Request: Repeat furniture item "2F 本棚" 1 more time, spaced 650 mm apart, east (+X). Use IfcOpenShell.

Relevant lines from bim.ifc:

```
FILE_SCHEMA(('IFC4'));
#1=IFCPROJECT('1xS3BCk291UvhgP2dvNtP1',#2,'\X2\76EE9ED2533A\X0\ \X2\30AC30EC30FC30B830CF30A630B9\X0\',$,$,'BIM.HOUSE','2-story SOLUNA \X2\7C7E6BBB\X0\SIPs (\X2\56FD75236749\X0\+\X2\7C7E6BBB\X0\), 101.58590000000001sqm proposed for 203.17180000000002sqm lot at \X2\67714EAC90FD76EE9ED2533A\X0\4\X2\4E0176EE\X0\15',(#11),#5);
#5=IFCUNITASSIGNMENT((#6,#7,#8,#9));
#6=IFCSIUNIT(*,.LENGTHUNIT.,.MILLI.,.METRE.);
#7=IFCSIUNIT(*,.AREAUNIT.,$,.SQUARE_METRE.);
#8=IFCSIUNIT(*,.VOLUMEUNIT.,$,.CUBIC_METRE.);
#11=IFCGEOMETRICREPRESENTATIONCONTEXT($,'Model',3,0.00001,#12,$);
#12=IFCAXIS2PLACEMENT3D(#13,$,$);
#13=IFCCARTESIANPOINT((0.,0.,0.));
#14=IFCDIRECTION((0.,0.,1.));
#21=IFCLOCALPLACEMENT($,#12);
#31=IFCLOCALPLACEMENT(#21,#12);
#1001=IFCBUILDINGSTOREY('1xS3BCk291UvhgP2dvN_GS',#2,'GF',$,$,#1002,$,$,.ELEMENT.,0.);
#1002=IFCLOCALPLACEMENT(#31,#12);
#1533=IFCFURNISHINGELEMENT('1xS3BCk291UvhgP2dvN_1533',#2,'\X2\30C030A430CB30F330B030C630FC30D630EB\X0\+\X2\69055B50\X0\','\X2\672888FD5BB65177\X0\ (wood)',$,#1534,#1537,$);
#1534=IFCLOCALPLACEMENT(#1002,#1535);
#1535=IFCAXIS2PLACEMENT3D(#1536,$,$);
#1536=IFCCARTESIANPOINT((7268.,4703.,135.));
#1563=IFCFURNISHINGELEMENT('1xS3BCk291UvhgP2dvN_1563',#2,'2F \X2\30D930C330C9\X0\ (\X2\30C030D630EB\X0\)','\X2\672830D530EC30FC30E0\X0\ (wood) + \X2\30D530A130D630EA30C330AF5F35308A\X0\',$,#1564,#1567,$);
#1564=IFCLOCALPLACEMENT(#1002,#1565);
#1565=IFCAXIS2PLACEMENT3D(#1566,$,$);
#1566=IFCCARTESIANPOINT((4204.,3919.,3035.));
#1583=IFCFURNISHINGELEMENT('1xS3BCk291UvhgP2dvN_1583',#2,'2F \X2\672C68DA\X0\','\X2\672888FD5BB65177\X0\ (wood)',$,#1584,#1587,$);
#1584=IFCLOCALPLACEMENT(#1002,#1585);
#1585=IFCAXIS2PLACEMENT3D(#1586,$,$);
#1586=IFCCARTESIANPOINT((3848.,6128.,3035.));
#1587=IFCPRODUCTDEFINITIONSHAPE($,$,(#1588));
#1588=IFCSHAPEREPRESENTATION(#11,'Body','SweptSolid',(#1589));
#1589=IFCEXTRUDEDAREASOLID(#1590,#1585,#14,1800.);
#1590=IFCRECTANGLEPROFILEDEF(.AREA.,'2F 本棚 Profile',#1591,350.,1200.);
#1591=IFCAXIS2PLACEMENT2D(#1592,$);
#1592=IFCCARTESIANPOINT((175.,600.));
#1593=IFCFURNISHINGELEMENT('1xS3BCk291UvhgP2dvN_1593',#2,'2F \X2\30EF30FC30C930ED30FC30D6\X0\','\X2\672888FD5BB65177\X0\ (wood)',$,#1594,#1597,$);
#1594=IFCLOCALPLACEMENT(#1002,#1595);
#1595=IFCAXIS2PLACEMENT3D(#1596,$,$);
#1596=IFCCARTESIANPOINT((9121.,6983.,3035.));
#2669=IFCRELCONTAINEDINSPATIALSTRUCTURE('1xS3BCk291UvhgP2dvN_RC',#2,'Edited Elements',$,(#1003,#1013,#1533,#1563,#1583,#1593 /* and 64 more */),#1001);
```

```python
import numpy as np
import ifcopenshell
import ifcopenshell.api.geometry
import ifcopenshell.api.root
import ifcopenshell.util.element
import ifcopenshell.util.placement

model = ifcopenshell.open("bim.ifc")


def reuse_history(source, copy):
    """copy_class also copies each property set's owner history, people and application; keep the originals."""
    for rel in copy.IsDefinedBy:
        if rel.is_a("IfcRelDefinesByProperties") and (history := rel.RelatingPropertyDefinition.OwnerHistory):
            rel.RelatingPropertyDefinition.OwnerHistory = source.OwnerHistory
            ifcopenshell.util.element.remove_deep2(model, history)


source = model.by_id(1583)
base = ifcopenshell.util.placement.get_local_placement(source.ObjectPlacement)
step = np.array([1.0, 0.0, 0.0]) * 650.0

for i in range(1, 2):
    copy = ifcopenshell.api.root.copy_class(model, product=source)
    copy.Representation = ifcopenshell.util.element.copy_deep(
        model, source.Representation, exclude=["IfcGeometricRepresentationContext", "IfcRepresentationMap"]
    )
    reuse_history(source, copy)
    matrix = base.copy()
    matrix[:3, 3] += i * step
    print("added at", matrix[:3, 3].round(3) + 0.0)
    ifcopenshell.api.geometry.edit_object_placement(model, product=copy, matrix=matrix, is_si=False)

model.write("bim_rev.ifc")
```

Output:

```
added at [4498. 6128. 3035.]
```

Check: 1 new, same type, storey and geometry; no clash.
